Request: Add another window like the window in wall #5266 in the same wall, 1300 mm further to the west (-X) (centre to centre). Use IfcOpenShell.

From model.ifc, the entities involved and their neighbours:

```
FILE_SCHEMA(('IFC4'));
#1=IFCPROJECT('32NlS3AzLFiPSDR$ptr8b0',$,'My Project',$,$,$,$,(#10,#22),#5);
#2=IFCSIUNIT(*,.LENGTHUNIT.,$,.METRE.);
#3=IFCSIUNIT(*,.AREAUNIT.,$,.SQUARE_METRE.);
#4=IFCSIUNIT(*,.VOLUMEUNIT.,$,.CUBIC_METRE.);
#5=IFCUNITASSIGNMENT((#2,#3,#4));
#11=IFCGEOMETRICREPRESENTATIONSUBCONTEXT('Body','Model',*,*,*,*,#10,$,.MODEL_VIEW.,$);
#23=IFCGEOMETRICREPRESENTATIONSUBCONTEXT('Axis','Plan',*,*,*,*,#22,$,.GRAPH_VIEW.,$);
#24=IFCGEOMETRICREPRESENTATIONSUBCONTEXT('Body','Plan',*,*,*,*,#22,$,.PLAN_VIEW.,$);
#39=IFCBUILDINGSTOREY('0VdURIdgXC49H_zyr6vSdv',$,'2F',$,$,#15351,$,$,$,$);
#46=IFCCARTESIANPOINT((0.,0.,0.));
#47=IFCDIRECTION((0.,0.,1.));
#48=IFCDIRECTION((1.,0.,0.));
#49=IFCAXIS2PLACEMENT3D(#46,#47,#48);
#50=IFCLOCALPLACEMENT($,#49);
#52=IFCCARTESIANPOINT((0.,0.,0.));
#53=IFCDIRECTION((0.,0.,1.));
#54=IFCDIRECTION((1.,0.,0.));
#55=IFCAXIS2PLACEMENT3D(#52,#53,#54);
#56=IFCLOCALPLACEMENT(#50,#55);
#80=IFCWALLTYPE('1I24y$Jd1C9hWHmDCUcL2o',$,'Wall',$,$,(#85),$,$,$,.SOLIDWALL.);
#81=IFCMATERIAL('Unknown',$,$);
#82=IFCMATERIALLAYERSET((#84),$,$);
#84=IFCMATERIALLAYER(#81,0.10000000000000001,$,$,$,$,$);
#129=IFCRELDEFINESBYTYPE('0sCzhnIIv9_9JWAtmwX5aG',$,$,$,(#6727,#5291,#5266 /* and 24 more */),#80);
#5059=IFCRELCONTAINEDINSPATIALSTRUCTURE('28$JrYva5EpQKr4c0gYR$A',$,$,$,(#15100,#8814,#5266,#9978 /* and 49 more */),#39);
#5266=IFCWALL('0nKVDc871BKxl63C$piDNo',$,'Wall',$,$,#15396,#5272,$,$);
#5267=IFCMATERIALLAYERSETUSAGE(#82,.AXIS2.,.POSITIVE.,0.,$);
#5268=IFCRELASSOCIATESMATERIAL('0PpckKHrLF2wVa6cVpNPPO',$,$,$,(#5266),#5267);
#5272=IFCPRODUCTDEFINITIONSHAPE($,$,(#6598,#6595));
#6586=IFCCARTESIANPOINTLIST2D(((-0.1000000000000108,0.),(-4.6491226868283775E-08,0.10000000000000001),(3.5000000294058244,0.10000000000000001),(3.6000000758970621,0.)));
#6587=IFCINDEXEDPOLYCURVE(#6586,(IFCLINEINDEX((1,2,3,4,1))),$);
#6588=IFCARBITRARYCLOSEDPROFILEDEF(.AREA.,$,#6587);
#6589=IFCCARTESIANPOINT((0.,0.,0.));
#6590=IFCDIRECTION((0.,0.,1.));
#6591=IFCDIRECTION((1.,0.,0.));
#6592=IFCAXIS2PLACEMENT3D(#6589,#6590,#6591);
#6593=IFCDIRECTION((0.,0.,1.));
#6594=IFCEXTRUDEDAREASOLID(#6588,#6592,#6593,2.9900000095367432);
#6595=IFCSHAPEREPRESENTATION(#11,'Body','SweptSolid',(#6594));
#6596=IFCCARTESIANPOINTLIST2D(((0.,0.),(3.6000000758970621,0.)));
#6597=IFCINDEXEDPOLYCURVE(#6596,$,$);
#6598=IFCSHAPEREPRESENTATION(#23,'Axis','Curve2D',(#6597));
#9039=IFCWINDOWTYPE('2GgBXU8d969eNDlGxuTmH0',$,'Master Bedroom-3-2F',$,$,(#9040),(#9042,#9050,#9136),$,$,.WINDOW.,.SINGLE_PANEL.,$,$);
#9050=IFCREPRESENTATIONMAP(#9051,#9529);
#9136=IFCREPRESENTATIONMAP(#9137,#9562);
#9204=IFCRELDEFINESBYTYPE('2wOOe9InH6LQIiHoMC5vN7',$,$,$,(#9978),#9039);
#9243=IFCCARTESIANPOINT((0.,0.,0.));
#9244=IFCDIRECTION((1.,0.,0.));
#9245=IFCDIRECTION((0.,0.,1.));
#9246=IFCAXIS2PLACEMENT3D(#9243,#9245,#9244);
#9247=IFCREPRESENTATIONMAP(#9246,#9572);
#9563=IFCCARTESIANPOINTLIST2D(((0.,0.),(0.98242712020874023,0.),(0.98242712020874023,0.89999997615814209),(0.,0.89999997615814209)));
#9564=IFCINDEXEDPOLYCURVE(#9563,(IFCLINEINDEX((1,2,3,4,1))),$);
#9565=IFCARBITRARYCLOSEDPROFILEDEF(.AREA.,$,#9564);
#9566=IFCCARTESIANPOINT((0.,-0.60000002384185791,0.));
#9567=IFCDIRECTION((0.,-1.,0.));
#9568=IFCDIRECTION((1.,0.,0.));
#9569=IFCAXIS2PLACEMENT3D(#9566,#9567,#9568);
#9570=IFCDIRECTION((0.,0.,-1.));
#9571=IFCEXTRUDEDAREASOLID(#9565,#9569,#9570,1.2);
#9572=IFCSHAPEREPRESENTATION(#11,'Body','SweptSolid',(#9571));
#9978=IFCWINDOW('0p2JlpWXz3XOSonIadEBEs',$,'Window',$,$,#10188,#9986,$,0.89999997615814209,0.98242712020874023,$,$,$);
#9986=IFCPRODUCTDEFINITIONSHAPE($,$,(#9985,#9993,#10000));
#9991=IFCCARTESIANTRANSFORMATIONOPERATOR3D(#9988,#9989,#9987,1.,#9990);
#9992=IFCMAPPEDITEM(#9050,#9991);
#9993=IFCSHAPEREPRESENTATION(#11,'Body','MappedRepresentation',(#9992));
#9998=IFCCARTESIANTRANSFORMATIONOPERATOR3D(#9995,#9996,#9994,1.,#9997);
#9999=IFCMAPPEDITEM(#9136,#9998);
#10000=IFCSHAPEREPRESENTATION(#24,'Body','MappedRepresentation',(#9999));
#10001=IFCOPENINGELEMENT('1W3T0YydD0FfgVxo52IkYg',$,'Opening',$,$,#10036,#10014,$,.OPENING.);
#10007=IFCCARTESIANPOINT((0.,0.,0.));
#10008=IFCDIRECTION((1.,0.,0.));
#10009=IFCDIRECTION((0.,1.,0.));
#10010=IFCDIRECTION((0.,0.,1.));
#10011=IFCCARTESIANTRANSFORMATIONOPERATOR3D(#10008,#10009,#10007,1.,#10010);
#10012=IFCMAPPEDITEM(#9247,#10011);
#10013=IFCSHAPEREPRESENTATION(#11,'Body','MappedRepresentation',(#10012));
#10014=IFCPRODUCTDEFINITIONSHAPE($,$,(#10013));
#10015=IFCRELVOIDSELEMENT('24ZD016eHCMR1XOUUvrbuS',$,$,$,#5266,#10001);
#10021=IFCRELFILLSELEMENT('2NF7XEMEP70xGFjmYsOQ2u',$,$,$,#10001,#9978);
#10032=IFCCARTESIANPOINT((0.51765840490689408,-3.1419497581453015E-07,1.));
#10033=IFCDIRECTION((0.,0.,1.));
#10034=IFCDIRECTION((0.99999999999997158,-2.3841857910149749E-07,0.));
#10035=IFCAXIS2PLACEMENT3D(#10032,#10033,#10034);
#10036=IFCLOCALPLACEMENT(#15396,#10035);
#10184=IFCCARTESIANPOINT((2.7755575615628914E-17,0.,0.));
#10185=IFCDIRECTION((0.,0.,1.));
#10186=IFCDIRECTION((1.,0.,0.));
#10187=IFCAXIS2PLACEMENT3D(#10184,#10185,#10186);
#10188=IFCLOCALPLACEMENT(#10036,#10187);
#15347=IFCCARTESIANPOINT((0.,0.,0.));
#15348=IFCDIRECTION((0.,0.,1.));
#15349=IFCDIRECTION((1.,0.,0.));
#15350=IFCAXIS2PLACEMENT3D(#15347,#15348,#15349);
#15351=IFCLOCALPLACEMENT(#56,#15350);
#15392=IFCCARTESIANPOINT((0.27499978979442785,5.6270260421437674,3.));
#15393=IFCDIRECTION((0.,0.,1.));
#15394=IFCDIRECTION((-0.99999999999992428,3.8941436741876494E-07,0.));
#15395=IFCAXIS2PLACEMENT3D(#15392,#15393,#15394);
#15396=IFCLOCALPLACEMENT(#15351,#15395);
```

```python
import ifcopenshell
import ifcopenshell.api.feature
import ifcopenshell.api.geometry
import ifcopenshell.api.root
import ifcopenshell.geom
import ifcopenshell.util.element
import ifcopenshell.util.placement
import ifcopenshell.util.shape
import ifcopenshell.util.unit

model = ifcopenshell.open("model.ifc")
unit_scale = ifcopenshell.util.unit.calculate_unit_scale(model)
settings = ifcopenshell.geom.settings()


def volume(element):
    """Net volume in cubic metres, openings subtracted."""
    shape = ifcopenshell.geom.create_shape(settings, element)
    return ifcopenshell.util.shape.get_volume(shape.geometry)


window = model.by_guid("0p2JlpWXz3XOSonIadEBEs")
opening = window.FillsVoids[0].RelatingOpeningElement
wall = opening.VoidsElements[0].RelatingBuildingElement
before = volume(wall)
shift = ifcopenshell.util.placement.get_local_placement(wall.ObjectPlacement)[:3, 0] * 1.3 / unit_scale

# copy_class copies the void relationship, type, container and properties, but no geometry.
new_opening = ifcopenshell.api.root.copy_class(model, product=opening)
new_opening.Representation = ifcopenshell.util.element.copy_deep(
    model, opening.Representation, exclude=["IfcGeometricRepresentationContext", "IfcRepresentationMap"]
)
new_window = ifcopenshell.api.root.copy_class(model, product=window)
new_window.Representation = ifcopenshell.util.element.copy_deep(
    model, window.Representation, exclude=["IfcGeometricRepresentationContext", "IfcRepresentationMap"]
)
ifcopenshell.api.feature.add_filling(model, opening=new_opening, element=new_window)

for old, new in ((opening, new_opening), (window, new_window)):
    matrix = ifcopenshell.util.placement.get_local_placement(old.ObjectPlacement)
    matrix[:3, 3] += shift
    ifcopenshell.api.geometry.edit_object_placement(model, product=new, matrix=matrix, is_si=False)

after = volume(wall)

print(f"wall volume {before:.3f} -> {after:.3f} m3")

model.write("model_updated.ifc")
```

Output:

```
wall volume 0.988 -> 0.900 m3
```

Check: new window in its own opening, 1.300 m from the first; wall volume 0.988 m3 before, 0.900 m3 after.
